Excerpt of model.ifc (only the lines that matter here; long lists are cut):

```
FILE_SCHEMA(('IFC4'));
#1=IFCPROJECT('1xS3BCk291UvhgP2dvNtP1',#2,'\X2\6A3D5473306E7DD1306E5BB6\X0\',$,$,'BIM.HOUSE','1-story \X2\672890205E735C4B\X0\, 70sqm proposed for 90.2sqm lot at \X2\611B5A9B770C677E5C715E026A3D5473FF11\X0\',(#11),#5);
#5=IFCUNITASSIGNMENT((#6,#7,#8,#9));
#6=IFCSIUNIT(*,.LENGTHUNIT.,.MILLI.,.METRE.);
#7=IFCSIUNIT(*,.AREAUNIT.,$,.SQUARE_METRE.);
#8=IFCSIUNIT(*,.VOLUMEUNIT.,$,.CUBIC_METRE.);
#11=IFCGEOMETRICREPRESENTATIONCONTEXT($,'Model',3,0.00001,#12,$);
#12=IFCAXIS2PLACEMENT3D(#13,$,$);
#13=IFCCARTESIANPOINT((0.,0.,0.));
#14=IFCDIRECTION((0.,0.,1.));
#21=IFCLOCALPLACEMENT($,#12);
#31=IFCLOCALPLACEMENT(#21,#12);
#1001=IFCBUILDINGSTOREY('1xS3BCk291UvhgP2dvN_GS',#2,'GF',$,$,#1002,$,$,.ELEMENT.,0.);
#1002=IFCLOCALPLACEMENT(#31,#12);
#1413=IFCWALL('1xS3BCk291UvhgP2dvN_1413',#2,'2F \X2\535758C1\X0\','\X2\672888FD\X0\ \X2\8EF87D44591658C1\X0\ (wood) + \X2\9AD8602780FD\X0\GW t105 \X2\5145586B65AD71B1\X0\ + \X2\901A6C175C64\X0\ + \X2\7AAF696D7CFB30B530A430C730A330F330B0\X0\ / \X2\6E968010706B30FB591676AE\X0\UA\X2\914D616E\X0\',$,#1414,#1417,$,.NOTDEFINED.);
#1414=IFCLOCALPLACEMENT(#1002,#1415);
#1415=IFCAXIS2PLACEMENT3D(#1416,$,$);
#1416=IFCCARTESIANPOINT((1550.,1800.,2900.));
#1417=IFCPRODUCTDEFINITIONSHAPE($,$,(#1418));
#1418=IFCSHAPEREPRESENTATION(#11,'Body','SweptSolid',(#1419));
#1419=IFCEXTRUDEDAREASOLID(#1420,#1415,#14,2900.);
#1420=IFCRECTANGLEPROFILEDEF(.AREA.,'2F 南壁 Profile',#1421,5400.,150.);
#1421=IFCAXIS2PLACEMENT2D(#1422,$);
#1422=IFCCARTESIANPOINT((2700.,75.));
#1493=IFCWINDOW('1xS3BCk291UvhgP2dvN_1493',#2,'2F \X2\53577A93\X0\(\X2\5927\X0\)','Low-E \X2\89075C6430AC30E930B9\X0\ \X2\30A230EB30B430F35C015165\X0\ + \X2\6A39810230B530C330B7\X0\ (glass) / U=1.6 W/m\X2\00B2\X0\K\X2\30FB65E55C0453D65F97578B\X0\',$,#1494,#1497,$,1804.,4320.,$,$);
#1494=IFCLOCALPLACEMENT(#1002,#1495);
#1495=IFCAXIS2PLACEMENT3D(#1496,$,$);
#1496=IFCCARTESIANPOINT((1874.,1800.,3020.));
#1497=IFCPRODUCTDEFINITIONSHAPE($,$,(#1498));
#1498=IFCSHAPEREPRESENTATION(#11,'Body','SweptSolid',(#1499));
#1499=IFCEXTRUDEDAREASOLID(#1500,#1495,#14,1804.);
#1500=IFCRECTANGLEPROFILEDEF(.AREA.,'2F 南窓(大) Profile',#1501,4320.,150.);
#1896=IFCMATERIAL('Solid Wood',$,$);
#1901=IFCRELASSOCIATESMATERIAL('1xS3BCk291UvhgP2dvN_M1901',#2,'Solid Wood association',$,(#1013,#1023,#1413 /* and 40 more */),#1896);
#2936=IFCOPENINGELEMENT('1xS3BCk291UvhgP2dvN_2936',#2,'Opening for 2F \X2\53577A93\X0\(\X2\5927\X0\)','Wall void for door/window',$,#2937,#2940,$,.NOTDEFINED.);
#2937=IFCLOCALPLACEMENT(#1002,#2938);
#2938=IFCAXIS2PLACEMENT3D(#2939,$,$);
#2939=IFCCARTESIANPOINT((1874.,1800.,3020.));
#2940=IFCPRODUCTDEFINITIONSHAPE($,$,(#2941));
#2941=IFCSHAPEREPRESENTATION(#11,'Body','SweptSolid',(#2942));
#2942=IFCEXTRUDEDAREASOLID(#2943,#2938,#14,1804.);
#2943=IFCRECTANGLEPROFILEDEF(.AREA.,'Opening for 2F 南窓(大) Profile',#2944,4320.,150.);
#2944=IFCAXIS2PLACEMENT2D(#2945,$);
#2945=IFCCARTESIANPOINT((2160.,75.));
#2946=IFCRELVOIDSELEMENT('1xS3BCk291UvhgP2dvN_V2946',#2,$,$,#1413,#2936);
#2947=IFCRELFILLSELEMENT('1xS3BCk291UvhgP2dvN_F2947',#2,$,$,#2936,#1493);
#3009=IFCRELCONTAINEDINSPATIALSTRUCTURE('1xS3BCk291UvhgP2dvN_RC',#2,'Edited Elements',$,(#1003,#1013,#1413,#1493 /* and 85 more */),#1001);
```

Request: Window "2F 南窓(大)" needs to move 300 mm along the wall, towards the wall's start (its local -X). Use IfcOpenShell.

```python
import ifcopenshell
import ifcopenshell.api.geometry
import ifcopenshell.util.placement

model = ifcopenshell.open("model.ifc")

window = model.by_id(1493)
opening = window.FillsVoids[0].RelatingOpeningElement
wall = opening.VoidsElements[0].RelatingBuildingElement

wall_matrix = ifcopenshell.util.placement.get_local_placement(wall.ObjectPlacement)
shift = wall_matrix[:3, 0] * -300.0
before = ifcopenshell.util.placement.get_local_placement(window.ObjectPlacement)[:3, 3].copy()

# The window is not placed relative to its opening, so move both.
for product in (opening, window):
    matrix = ifcopenshell.util.placement.get_local_placement(product.ObjectPlacement)
    matrix[:3, 3] += shift
    ifcopenshell.api.geometry.edit_object_placement(model, product=product, matrix=matrix, is_si=False)

after = ifcopenshell.util.placement.get_local_placement(window.ObjectPlacement)[:3, 3]
print("window moved by", (after - before).round(3) + 0.0)

model.write("model_updated.ifc")
```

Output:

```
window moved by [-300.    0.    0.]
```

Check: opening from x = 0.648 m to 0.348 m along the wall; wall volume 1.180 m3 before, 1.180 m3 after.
